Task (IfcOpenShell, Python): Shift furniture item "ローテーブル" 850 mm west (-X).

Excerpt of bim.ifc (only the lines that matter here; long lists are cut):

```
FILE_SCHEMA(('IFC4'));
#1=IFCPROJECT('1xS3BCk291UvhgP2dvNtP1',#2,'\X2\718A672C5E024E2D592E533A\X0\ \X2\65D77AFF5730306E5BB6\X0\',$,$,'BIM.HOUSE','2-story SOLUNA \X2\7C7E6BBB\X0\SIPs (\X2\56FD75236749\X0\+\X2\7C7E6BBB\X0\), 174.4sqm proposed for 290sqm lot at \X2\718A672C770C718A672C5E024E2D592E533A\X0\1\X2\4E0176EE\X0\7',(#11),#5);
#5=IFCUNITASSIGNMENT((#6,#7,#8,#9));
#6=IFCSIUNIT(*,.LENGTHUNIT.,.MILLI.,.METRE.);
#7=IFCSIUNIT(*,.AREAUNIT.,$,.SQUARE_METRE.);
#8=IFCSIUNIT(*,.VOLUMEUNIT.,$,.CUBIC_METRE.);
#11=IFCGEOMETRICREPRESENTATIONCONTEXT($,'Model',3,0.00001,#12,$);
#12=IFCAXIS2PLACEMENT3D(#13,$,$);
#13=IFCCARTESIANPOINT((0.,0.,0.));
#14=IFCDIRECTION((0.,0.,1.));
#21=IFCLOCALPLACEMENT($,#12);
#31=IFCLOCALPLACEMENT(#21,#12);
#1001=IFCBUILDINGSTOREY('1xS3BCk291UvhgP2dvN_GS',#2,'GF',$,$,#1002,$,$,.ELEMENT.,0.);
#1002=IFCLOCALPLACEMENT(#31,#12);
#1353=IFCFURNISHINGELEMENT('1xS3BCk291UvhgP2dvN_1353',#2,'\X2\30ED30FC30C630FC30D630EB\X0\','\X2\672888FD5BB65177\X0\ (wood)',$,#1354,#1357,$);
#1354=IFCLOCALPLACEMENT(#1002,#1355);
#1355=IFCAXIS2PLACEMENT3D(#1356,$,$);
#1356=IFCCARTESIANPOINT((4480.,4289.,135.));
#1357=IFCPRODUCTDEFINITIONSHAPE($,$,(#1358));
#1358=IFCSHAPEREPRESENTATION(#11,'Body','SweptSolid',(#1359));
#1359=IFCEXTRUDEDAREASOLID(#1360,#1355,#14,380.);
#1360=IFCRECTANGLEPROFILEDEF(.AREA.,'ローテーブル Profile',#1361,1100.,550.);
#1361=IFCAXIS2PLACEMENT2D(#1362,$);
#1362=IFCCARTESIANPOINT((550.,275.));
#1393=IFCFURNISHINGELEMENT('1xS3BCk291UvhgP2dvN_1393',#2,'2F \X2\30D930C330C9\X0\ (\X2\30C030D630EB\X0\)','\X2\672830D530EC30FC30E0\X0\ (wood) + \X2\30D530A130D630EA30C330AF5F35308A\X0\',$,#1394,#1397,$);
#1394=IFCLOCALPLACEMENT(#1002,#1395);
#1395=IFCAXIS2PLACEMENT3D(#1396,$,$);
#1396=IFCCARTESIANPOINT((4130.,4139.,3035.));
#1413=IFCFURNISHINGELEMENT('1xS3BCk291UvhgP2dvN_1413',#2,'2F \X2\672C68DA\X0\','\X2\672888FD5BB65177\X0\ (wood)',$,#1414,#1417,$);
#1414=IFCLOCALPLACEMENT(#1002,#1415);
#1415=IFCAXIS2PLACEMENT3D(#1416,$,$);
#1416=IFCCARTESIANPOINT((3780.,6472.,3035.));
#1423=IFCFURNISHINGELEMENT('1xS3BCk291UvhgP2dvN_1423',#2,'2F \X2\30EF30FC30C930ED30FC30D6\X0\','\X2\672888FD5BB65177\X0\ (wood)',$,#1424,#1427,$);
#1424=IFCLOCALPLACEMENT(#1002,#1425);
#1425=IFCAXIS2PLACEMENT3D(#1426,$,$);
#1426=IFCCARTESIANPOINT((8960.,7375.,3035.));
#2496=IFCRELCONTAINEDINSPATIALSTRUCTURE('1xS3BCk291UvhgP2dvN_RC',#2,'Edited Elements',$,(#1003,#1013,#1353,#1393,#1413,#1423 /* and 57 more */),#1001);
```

```python
import ifcopenshell
import ifcopenshell.api.geometry
import ifcopenshell.util.placement

model = ifcopenshell.open("bim.ifc")

item = model.by_guid("1xS3BCk291UvhgP2dvN_1353")
matrix = ifcopenshell.util.placement.get_local_placement(item.ObjectPlacement)
matrix[0, 3] -= 850.0
ifcopenshell.api.geometry.edit_object_placement(model, product=item, matrix=matrix, is_si=False)

print(ifcopenshell.util.placement.get_local_placement(item.ObjectPlacement).round(3) + 0.0)

model.write("bim_v2.ifc")
```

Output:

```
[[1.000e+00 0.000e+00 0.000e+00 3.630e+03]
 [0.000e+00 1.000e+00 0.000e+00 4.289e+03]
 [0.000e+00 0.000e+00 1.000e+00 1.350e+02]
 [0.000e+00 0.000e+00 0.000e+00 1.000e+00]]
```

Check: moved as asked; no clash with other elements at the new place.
